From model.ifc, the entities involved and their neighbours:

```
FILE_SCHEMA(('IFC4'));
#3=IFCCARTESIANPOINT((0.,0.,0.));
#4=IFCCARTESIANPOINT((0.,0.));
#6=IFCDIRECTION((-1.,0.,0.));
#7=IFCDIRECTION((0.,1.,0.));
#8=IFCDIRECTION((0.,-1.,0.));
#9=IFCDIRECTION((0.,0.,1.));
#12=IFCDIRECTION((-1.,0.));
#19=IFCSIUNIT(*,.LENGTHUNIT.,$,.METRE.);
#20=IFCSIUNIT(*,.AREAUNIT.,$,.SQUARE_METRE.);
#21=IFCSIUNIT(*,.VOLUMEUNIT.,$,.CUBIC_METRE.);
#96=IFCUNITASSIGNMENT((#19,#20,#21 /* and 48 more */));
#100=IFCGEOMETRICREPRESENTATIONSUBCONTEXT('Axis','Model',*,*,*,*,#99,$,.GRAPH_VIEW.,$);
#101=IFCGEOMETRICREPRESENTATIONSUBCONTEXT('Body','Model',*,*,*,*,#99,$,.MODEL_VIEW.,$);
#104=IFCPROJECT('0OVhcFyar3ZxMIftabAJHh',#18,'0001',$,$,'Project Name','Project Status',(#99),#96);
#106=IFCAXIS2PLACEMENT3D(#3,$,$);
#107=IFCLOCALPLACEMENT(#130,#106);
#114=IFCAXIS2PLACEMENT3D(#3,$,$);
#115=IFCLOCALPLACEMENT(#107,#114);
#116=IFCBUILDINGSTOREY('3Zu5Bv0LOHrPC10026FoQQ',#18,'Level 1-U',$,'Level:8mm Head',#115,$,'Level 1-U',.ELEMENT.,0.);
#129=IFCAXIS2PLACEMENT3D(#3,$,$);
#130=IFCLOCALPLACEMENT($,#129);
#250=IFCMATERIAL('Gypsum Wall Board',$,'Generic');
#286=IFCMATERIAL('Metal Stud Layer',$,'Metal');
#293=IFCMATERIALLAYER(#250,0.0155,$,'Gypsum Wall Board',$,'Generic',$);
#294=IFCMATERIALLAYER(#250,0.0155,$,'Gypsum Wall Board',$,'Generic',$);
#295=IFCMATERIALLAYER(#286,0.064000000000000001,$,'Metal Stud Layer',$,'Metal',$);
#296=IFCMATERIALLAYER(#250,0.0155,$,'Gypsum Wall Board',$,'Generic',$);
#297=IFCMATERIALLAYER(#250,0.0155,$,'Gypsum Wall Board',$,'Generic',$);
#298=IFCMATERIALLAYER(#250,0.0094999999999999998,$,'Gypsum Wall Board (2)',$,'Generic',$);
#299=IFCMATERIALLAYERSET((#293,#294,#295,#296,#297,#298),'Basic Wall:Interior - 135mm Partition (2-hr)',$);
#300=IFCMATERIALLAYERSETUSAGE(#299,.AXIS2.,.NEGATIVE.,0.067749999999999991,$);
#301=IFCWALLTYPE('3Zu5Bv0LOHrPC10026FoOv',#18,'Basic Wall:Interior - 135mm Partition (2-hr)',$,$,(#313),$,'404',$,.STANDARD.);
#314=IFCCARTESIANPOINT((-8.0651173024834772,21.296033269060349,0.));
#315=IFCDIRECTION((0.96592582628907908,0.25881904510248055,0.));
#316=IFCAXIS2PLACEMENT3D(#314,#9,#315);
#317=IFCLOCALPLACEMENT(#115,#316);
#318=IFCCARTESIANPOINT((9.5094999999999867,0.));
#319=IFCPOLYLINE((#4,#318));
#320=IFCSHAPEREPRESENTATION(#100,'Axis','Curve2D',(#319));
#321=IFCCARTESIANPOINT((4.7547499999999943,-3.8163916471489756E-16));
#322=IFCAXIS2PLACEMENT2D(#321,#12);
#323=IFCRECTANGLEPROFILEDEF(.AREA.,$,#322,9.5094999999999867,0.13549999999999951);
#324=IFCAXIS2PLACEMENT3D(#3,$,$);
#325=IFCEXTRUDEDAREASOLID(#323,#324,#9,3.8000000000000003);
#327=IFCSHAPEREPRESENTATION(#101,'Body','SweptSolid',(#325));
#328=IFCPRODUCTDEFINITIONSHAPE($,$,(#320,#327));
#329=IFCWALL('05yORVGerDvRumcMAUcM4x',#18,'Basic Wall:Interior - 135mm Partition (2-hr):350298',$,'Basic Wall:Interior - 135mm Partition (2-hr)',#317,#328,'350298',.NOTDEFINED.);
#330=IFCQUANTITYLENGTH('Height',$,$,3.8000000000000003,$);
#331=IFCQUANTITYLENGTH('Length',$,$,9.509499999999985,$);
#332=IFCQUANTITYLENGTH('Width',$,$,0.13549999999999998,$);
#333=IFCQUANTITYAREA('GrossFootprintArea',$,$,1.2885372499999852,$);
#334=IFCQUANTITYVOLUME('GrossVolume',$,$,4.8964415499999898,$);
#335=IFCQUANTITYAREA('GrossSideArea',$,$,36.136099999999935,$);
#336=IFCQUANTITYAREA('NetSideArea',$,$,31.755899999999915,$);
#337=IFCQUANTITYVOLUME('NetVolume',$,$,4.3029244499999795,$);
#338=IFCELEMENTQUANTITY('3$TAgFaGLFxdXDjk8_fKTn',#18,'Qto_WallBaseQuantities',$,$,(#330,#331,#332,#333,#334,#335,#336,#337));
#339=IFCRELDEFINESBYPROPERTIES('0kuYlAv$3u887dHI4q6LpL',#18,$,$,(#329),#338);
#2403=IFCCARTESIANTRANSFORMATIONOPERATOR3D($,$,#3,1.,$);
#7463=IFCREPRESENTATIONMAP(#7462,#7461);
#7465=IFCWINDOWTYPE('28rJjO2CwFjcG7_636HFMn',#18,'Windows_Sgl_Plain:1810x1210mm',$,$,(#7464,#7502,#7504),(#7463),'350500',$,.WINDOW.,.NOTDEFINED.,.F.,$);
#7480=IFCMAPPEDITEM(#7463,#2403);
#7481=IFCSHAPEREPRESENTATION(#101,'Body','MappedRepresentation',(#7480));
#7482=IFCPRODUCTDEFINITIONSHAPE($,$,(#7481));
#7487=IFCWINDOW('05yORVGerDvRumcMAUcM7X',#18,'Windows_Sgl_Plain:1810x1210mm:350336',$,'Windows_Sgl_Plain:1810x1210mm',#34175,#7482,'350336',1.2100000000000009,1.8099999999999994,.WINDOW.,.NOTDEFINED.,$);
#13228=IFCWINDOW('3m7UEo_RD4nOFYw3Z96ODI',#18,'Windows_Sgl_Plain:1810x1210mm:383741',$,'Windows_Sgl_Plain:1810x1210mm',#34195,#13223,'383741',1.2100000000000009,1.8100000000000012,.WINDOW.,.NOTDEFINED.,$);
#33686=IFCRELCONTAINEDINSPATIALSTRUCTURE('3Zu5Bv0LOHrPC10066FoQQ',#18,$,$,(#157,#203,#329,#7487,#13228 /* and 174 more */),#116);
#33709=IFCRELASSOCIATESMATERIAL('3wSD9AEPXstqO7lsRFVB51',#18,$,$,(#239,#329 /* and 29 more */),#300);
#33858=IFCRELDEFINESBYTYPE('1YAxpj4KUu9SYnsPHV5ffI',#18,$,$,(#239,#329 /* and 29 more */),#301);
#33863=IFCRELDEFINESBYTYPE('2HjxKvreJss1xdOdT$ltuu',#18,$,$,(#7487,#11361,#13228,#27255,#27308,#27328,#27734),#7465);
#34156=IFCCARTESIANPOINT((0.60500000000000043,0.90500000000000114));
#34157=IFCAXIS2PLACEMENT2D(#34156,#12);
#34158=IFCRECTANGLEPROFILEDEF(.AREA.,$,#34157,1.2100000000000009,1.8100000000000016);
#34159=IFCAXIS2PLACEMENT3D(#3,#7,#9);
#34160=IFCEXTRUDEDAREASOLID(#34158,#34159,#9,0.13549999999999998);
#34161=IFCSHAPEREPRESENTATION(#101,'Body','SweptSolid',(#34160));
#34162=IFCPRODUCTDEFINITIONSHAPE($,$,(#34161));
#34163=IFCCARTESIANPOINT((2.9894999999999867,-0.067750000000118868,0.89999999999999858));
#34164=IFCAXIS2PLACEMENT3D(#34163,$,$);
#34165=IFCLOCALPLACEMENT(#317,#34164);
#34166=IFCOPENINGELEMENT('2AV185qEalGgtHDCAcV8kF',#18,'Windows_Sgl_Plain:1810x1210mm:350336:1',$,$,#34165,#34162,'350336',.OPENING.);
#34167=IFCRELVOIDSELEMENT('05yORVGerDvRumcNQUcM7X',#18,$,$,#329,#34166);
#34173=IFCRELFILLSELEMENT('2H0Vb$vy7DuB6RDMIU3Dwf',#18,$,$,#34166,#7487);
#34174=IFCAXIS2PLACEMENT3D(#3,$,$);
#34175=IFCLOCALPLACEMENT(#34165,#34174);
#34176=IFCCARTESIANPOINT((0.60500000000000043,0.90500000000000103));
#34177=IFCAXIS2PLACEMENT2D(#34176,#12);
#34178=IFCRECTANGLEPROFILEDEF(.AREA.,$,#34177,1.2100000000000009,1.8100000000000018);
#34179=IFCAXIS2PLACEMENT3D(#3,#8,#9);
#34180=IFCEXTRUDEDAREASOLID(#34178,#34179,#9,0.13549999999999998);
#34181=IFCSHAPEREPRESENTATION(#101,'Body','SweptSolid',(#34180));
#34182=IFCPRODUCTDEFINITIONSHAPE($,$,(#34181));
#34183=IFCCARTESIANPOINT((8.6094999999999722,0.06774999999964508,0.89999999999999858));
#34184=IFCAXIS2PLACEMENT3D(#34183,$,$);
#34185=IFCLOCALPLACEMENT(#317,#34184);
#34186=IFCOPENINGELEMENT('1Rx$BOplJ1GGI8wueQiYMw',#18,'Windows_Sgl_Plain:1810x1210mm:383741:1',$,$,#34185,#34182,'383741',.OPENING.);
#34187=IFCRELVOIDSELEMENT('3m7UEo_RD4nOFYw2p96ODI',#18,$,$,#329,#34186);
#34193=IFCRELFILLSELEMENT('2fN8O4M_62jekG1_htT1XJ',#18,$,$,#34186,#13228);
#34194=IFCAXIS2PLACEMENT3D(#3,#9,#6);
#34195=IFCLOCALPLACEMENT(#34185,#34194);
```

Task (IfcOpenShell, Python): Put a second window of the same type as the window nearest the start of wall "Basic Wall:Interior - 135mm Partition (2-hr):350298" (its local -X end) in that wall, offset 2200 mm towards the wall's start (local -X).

```python
import ifcopenshell
import ifcopenshell.api.feature
import ifcopenshell.api.geometry
import ifcopenshell.api.pset
import ifcopenshell.api.root
import ifcopenshell.geom
import ifcopenshell.util.element
import ifcopenshell.util.placement
import ifcopenshell.util.shape
import ifcopenshell.util.unit

model = ifcopenshell.open("model.ifc")
unit_scale = ifcopenshell.util.unit.calculate_unit_scale(model)
area_scale = ifcopenshell.util.unit.calculate_unit_scale(model, "AREAUNIT")
volume_scale = ifcopenshell.util.unit.calculate_unit_scale(model, "VOLUMEUNIT")
settings = ifcopenshell.geom.settings()


def volume(element):
    """Net volume in cubic metres, openings subtracted."""
    shape = ifcopenshell.geom.create_shape(settings, element)
    return ifcopenshell.util.shape.get_volume(shape.geometry)


def reuse_history(source, copy):
    """copy_class also copies each property set's owner history, people and application; keep the originals."""
    for rel in copy.IsDefinedBy:
        if rel.is_a("IfcRelDefinesByProperties") and (history := rel.RelatingPropertyDefinition.OwnerHistory):
            rel.RelatingPropertyDefinition.OwnerHistory = source.OwnerHistory
            ifcopenshell.util.element.remove_deep2(model, history)


window = model.by_id(7487)
opening = window.FillsVoids[0].RelatingOpeningElement
wall = opening.VoidsElements[0].RelatingBuildingElement
before = volume(wall)
shift = ifcopenshell.util.placement.get_local_placement(wall.ObjectPlacement)[:3, 0] * -2.2 / unit_scale

# copy_class copies the void relationship, type, container and properties, but no geometry.
new_opening = ifcopenshell.api.root.copy_class(model, product=opening)
new_opening.Representation = ifcopenshell.util.element.copy_deep(
    model, opening.Representation, exclude=["IfcGeometricRepresentationContext", "IfcRepresentationMap"]
)
new_opening.Name = "Windows_Sgl_Plain:1810x1210mm"
new_opening.Tag = None
reuse_history(opening, new_opening)
new_window = ifcopenshell.api.root.copy_class(model, product=window)
new_window.Representation = ifcopenshell.util.element.copy_deep(
    model, window.Representation, exclude=["IfcGeometricRepresentationContext", "IfcRepresentationMap"]
)
new_window.Name = "Windows_Sgl_Plain:1810x1210mm"
new_window.Tag = None
reuse_history(window, new_window)
ifcopenshell.api.feature.add_filling(model, opening=new_opening, element=new_window)

for old, new in ((opening, new_opening), (window, new_window)):
    matrix = ifcopenshell.util.placement.get_local_placement(old.ObjectPlacement)
    matrix[:3, 3] += shift
    ifcopenshell.api.geometry.edit_object_placement(model, product=new, matrix=matrix, is_si=False)

after = volume(wall)
thickness = 0.1355  # wall thickness in metres

# Update the wall's stored quantities.
qto = model.by_id(ifcopenshell.util.element.get_pset(wall, "Qto_WallBaseQuantities", should_inherit=False)["id"])
ifcopenshell.api.pset.edit_qto(model, qto=qto, properties={
    "NetSideArea": after / thickness / area_scale,
    "NetVolume": after / volume_scale,
})

print(f"wall volume {before:.3f} -> {after:.3f} m3")

model.write("model-out.ifc")
```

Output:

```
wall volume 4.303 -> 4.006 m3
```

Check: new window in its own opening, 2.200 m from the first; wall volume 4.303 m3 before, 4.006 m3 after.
